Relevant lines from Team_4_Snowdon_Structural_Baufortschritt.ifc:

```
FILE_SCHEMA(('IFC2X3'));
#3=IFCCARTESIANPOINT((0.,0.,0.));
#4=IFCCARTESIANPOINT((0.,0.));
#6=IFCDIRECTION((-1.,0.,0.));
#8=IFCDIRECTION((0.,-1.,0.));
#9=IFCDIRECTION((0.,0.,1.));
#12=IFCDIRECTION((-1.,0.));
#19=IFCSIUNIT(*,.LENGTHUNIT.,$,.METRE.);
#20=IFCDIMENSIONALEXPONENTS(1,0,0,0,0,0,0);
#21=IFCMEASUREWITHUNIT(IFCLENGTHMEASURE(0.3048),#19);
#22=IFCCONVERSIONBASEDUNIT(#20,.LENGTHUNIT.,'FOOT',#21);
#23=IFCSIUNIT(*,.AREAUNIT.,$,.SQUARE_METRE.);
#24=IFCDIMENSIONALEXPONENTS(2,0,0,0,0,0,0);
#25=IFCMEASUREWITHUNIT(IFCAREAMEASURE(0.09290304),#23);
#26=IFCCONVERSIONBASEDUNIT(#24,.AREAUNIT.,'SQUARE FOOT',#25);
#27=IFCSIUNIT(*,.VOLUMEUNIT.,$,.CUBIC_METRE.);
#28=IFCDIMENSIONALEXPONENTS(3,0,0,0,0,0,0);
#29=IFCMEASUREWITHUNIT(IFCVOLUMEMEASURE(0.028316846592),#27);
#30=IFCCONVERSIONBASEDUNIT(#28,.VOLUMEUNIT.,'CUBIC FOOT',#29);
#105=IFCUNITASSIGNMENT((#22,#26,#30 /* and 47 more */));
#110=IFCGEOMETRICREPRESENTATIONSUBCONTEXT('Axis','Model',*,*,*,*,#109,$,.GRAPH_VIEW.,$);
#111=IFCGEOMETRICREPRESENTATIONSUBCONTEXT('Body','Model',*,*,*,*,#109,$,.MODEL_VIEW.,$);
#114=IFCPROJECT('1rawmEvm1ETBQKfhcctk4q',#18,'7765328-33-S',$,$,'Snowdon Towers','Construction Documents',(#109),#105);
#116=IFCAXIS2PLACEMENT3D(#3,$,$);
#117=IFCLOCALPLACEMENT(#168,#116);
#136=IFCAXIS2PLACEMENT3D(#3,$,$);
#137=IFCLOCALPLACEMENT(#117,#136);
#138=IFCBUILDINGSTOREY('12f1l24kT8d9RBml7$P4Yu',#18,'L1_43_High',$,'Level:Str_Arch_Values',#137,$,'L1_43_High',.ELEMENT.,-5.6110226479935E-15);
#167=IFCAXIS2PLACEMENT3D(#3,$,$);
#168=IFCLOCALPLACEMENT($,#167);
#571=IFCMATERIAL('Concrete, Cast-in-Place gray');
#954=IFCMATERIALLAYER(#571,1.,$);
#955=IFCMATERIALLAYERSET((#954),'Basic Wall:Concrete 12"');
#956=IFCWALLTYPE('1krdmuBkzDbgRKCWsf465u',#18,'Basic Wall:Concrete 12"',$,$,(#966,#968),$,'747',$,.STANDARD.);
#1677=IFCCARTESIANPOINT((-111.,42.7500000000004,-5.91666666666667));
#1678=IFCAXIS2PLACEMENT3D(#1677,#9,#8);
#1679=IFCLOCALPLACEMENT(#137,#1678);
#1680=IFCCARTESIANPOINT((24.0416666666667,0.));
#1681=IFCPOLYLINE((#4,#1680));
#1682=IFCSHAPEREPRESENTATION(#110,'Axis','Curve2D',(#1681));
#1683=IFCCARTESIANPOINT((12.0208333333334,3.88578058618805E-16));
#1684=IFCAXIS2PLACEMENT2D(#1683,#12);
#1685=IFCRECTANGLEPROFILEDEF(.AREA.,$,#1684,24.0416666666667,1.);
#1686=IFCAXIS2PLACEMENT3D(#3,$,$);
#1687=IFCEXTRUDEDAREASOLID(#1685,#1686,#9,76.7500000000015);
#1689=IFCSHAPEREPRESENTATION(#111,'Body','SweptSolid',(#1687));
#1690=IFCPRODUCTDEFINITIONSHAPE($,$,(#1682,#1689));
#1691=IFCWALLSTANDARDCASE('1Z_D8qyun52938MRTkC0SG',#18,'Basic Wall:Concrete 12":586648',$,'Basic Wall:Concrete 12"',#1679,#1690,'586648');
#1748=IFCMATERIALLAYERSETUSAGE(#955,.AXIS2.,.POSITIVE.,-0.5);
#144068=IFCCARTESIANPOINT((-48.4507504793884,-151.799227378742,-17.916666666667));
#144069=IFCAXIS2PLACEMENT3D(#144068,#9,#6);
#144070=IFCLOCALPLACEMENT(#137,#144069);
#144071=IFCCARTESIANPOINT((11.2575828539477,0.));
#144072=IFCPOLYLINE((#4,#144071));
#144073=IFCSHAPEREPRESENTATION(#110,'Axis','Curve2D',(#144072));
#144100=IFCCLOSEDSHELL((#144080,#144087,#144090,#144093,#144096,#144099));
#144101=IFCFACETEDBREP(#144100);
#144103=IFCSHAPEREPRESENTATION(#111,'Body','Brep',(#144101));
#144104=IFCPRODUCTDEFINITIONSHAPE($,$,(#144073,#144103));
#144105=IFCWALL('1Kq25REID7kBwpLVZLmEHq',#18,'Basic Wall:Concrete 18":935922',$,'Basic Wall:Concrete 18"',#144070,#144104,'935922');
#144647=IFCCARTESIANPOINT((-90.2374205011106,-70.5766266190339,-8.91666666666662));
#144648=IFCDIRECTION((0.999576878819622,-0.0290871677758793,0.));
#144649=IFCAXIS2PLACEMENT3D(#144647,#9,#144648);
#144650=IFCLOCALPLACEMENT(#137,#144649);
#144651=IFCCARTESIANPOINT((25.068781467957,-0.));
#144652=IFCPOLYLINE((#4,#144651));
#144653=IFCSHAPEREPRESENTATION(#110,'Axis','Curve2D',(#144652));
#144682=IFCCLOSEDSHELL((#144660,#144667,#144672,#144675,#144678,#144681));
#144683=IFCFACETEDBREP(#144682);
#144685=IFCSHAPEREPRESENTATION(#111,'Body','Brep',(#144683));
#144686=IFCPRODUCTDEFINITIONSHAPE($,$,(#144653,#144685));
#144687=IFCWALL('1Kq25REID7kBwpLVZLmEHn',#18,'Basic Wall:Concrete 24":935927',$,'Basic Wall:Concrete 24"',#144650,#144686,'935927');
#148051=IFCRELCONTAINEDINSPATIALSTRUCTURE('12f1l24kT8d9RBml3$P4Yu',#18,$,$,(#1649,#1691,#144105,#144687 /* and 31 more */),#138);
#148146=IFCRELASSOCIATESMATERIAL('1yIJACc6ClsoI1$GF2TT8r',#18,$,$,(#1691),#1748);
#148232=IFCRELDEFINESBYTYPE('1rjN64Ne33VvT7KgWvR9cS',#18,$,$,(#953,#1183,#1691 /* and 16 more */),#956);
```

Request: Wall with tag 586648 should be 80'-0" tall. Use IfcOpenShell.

```python
import ifcopenshell
import ifcopenshell.geom
import ifcopenshell.util.representation
import ifcopenshell.util.shape
import ifcopenshell.util.unit

model = ifcopenshell.open("Team_4_Snowdon_Structural_Baufortschritt.ifc")
unit_scale = ifcopenshell.util.unit.calculate_unit_scale(model)
settings = ifcopenshell.geom.settings()


def volume(element):
    """Net volume in cubic metres, openings subtracted."""
    shape = ifcopenshell.geom.create_shape(settings, element)
    return ifcopenshell.util.shape.get_volume(shape.geometry)


wall = model.by_guid("1Z_D8qyun52938MRTkC0SG")
before = volume(wall)

body = ifcopenshell.util.representation.get_representation(wall, "Model", "Body")
solid = body.Items[0]
old_height = solid.Depth
solid.Depth = 960 * 0.0254 / unit_scale
after = volume(wall)

print(f"height {old_height:g} -> {solid.Depth:g}, volume {before:.3f} -> {after:.3f} m3")

model.write("Team_4_Snowdon_Structural_Baufortschritt_rev.ifc")
```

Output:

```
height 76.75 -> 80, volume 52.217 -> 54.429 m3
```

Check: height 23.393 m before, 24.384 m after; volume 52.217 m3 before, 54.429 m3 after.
